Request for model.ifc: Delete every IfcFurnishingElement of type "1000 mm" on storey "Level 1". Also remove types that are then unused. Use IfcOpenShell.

First a look at what the model holds.

```python
import ifcopenshell
import ifcopenshell.util.element

model = ifcopenshell.open("model.ifc")
print(model.schema)
storey = next(s for s in model.by_type("IfcBuildingStorey") if s.Name == "Level 1")
furniture = [e for e in ifcopenshell.util.element.get_decomposition(storey) if e.is_a("IfcFurnishingElement")]
seen = {}
for e in furniture:
    element_type = ifcopenshell.util.element.get_type(e)
    name = element_type.Name if element_type not in (None, e) else None
    seen[name] = seen.get(name, 0) + 1
for name, count in sorted(seen.items(), key=str):
    print(count, "x", name)
```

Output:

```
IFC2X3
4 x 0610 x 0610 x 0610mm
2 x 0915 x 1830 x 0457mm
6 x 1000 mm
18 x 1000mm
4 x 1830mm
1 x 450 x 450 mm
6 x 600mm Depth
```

```python
import ifcopenshell
import ifcopenshell.api.root
import ifcopenshell.util.element

model = ifcopenshell.open("model.ifc")

storey = next(s for s in model.by_type("IfcBuildingStorey") if s.Name == "Level 1")
furniture = [e for e in ifcopenshell.util.element.get_decomposition(storey) if e.is_a("IfcFurnishingElement")]
targets = [e for e in furniture if (t := ifcopenshell.util.element.get_type(e)) not in (None, e) and t.Name == "1000 mm"]
types = {ifcopenshell.util.element.get_type(e) for e in targets} - {None, *targets}

for e in targets:
    ifcopenshell.api.root.remove_product(model, product=e)
print(len(targets), "removed")

unused = [t for t in types if not ifcopenshell.util.element.get_types(t)]
for t in unused:
    ifcopenshell.api.root.remove_product(model, product=t)
print(len(unused), "unused types removed")

model.write("model-out.ifc")
```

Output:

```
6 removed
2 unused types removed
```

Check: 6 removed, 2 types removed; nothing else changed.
